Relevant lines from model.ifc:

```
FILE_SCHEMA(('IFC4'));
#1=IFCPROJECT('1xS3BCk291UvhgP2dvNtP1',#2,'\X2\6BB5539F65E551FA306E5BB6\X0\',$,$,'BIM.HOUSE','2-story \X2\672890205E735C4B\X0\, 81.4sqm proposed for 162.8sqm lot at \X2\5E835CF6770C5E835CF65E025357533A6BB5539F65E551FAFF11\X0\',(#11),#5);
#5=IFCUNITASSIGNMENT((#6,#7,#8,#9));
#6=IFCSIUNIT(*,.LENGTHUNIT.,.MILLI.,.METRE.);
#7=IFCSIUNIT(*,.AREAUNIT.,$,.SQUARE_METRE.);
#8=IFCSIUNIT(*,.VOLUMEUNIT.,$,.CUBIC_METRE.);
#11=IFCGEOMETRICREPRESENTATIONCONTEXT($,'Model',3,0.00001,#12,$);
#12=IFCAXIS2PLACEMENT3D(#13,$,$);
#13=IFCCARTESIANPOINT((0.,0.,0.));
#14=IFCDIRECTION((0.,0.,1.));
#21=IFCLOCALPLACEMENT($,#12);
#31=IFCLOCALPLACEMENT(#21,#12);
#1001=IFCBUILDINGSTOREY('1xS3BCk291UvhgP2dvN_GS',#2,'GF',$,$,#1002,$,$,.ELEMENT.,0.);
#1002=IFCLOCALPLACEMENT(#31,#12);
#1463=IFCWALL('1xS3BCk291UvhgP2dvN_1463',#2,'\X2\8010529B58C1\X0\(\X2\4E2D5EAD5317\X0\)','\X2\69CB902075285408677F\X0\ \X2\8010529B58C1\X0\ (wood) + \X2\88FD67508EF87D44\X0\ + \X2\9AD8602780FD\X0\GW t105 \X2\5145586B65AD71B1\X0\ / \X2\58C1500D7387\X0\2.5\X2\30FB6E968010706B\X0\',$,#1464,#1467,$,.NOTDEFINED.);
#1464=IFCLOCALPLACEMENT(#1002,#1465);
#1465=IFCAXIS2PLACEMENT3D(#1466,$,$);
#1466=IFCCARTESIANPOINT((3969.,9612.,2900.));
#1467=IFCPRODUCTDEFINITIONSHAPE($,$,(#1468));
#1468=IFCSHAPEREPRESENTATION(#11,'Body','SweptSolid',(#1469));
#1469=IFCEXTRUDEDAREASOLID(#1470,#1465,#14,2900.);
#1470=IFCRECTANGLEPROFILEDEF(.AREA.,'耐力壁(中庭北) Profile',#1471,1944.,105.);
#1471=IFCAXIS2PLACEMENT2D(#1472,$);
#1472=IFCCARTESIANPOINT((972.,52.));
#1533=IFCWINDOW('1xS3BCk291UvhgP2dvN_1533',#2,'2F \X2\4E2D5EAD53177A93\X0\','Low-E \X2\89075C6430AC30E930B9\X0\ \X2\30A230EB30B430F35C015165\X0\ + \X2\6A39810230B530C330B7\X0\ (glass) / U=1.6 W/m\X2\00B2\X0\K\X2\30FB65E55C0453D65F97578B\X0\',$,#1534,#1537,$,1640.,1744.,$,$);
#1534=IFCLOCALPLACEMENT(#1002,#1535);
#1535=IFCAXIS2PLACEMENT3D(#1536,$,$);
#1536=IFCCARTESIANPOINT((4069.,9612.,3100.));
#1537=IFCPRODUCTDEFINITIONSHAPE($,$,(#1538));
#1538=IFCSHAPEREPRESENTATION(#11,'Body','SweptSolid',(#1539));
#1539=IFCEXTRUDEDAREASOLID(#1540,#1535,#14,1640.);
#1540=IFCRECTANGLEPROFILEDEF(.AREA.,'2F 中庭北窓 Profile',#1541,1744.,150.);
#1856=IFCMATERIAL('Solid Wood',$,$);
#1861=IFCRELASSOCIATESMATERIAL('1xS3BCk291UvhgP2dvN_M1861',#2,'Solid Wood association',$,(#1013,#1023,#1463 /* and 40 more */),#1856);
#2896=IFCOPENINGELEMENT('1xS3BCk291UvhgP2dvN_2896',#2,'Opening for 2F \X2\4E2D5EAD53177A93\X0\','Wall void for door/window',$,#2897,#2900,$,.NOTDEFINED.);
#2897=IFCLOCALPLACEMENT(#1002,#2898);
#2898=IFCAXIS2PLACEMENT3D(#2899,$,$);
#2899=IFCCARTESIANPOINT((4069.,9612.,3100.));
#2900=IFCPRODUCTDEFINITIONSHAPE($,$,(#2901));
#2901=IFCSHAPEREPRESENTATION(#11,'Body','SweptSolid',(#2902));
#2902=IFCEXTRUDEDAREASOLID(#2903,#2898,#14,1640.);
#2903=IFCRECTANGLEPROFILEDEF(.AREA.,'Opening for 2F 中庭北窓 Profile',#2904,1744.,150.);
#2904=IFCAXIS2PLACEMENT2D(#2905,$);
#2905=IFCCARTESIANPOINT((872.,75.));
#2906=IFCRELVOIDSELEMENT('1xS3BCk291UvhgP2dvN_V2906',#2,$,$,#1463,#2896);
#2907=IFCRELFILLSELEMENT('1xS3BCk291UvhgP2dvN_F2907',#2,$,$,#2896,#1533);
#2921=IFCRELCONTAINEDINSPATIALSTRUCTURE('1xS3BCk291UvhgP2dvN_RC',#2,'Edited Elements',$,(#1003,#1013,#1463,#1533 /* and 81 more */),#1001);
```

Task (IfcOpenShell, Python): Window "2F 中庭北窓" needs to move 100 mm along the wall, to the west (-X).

```python
import ifcopenshell
import ifcopenshell.api.geometry
import ifcopenshell.util.placement

model = ifcopenshell.open("model.ifc")

window = model.by_guid("1xS3BCk291UvhgP2dvN_1533")
opening = window.FillsVoids[0].RelatingOpeningElement
wall = opening.VoidsElements[0].RelatingBuildingElement

wall_matrix = ifcopenshell.util.placement.get_local_placement(wall.ObjectPlacement)
shift = wall_matrix[:3, 0] * -100.0
before = ifcopenshell.util.placement.get_local_placement(window.ObjectPlacement)[:3, 3].copy()

# The window is not placed relative to its opening, so move both.
for product in (opening, window):
    matrix = ifcopenshell.util.placement.get_local_placement(product.ObjectPlacement)
    matrix[:3, 3] += shift
    ifcopenshell.api.geometry.edit_object_placement(model, product=product, matrix=matrix, is_si=False)

after = ifcopenshell.util.placement.get_local_placement(window.ObjectPlacement)[:3, 3]
print("window moved by", (after - before).round(3) + 0.0)

model.write("model_rev.ifc")
```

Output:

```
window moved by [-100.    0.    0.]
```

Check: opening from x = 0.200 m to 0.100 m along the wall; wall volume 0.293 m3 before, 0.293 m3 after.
